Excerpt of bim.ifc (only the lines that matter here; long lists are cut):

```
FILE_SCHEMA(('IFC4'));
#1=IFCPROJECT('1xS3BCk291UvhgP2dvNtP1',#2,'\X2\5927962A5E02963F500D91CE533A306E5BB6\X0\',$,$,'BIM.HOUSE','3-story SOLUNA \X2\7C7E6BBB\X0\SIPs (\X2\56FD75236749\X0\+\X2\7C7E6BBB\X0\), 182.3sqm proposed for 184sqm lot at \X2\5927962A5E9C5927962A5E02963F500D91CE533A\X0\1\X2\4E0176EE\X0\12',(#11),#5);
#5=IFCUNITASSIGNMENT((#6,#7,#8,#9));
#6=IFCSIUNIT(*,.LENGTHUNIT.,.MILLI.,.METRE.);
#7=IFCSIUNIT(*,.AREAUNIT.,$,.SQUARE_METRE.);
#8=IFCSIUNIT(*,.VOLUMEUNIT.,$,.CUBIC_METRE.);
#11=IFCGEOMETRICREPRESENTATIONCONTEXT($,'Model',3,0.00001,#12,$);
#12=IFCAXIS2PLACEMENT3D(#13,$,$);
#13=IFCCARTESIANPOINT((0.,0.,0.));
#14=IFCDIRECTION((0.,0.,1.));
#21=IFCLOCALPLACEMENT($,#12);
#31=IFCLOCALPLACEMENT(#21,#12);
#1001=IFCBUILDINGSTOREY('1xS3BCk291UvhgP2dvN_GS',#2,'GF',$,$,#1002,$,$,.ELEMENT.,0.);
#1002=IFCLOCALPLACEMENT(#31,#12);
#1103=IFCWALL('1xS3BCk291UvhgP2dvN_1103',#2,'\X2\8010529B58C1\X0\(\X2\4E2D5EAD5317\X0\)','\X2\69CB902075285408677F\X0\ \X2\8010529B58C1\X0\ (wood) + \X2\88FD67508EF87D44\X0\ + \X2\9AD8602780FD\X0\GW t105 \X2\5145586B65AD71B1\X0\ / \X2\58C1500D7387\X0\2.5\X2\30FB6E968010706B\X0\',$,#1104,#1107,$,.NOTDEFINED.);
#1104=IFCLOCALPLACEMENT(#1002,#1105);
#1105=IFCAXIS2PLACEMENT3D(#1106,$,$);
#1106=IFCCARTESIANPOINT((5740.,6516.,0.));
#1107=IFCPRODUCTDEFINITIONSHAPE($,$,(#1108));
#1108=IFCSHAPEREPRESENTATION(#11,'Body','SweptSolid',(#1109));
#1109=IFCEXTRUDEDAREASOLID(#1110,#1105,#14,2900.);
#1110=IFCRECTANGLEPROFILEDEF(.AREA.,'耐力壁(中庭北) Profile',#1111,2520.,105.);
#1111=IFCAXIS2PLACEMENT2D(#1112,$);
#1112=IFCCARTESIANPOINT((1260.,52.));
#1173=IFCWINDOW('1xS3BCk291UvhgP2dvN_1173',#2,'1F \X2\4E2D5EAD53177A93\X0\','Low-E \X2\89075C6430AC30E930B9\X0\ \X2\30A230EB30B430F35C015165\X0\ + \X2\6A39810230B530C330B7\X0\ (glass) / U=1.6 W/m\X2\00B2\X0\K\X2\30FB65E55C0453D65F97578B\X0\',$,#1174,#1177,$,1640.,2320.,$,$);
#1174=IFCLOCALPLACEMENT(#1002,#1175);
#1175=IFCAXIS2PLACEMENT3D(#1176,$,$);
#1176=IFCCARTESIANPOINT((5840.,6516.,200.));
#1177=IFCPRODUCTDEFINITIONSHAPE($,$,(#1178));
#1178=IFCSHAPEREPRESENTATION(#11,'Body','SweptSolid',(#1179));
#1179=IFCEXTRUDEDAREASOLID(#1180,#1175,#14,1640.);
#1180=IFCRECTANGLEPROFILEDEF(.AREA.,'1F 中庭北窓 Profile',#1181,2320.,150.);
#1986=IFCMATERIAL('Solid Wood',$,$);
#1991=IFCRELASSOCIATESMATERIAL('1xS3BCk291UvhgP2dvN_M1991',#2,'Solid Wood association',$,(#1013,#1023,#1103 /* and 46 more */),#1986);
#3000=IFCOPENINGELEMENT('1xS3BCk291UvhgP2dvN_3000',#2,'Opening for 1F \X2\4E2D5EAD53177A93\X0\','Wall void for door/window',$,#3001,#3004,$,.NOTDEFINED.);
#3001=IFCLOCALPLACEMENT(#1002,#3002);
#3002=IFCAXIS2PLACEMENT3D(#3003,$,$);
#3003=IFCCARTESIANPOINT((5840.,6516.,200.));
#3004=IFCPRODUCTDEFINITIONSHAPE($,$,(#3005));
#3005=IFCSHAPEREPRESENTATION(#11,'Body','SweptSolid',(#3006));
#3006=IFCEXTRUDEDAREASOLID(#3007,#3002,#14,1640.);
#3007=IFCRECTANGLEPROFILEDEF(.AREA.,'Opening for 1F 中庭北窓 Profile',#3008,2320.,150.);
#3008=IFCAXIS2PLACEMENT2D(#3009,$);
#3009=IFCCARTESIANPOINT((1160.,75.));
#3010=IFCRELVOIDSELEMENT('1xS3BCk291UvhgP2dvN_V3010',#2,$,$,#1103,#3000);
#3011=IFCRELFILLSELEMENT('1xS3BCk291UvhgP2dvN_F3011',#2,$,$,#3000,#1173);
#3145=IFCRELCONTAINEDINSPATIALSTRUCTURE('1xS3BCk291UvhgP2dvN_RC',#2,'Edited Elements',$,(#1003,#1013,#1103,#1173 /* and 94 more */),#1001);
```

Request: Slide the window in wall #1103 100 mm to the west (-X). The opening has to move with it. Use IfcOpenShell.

```python
import ifcopenshell
import ifcopenshell.api.geometry
import ifcopenshell.util.placement

model = ifcopenshell.open("bim.ifc")

window = model.by_guid("1xS3BCk291UvhgP2dvN_1173")
opening = window.FillsVoids[0].RelatingOpeningElement
wall = opening.VoidsElements[0].RelatingBuildingElement

wall_matrix = ifcopenshell.util.placement.get_local_placement(wall.ObjectPlacement)
shift = wall_matrix[:3, 0] * -100.0
before = ifcopenshell.util.placement.get_local_placement(window.ObjectPlacement)[:3, 3].copy()

# The window is not placed relative to its opening, so move both.
for product in (opening, window):
    matrix = ifcopenshell.util.placement.get_local_placement(product.ObjectPlacement)
    matrix[:3, 3] += shift
    ifcopenshell.api.geometry.edit_object_placement(model, product=product, matrix=matrix, is_si=False)

after = ifcopenshell.util.placement.get_local_placement(window.ObjectPlacement)[:3, 3]
print("window moved by", (after - before).round(3) + 0.0)

model.write("bim_edited.ifc")
```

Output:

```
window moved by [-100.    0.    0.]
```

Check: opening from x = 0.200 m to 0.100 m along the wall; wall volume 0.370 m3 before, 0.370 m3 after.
